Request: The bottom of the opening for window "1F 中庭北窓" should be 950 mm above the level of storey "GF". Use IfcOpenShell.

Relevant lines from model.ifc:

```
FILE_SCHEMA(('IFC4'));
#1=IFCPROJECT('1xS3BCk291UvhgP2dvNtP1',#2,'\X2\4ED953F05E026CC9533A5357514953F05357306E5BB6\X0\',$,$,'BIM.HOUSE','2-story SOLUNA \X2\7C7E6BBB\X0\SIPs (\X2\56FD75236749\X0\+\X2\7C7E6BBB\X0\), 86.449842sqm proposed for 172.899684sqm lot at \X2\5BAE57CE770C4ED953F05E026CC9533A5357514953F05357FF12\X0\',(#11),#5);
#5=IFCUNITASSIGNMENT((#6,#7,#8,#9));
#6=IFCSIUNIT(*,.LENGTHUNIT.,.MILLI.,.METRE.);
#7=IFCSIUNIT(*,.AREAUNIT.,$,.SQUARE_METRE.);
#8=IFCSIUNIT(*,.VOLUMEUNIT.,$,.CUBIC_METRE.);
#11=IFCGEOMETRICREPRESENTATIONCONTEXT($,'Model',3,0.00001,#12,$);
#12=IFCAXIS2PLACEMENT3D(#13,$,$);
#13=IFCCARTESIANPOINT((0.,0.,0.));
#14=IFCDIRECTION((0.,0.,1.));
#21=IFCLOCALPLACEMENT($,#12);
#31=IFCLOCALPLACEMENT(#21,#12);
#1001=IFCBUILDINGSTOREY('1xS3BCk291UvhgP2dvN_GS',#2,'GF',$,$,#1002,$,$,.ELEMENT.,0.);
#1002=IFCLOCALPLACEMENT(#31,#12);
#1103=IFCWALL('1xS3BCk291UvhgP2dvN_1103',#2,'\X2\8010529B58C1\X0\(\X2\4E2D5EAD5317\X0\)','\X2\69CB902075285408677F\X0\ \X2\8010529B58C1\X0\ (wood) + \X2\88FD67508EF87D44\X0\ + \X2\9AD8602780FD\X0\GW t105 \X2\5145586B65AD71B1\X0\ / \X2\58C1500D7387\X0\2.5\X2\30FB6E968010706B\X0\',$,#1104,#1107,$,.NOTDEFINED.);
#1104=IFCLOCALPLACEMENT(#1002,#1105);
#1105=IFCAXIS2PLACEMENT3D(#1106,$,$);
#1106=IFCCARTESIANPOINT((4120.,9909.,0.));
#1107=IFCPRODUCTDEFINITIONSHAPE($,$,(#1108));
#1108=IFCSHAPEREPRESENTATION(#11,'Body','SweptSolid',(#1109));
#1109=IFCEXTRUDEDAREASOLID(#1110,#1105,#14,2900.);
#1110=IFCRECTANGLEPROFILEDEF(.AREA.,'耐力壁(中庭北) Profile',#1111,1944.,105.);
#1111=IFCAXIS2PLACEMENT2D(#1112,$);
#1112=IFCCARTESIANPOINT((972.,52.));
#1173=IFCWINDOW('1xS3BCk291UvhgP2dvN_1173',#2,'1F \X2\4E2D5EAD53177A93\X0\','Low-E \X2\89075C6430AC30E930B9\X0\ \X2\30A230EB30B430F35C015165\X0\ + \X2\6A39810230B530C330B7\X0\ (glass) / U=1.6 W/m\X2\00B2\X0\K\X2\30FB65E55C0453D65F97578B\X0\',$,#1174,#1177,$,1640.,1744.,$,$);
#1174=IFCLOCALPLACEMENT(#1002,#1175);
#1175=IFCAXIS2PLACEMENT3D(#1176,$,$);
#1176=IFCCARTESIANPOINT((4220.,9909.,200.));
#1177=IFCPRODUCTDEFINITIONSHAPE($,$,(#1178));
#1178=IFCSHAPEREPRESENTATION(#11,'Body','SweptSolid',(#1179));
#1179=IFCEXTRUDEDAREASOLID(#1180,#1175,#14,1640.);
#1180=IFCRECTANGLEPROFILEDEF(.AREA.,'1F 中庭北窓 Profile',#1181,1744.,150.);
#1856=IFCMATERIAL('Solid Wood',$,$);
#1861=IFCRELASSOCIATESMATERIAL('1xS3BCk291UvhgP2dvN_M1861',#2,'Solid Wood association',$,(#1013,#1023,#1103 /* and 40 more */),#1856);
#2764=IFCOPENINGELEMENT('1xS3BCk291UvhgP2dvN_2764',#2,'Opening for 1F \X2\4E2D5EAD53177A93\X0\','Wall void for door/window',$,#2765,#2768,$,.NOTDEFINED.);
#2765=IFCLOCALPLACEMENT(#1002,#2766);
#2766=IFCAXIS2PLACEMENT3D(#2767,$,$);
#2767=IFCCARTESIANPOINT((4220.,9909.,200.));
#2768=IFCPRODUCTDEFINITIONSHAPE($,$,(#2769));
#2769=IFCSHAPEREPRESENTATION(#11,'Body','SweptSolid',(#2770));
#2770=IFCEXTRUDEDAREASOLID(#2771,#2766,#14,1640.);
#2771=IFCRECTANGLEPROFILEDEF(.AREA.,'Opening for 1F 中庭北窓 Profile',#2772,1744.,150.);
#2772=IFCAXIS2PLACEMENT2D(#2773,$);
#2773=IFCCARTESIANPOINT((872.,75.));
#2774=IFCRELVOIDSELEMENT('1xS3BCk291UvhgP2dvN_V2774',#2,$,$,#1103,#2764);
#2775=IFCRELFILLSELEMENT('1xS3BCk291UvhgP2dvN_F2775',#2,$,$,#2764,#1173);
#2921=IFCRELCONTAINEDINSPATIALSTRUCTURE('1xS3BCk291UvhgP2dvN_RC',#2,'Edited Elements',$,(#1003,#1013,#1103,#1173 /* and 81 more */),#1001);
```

```python
import numpy as np
import ifcopenshell
import ifcopenshell.api.geometry
import ifcopenshell.geom
import ifcopenshell.util.element
import ifcopenshell.util.placement
import ifcopenshell.util.shape
import ifcopenshell.util.unit

model = ifcopenshell.open("model.ifc")
unit_scale = ifcopenshell.util.unit.calculate_unit_scale(model)

window = model.by_guid("1xS3BCk291UvhgP2dvN_1173")
opening = window.FillsVoids[0].RelatingOpeningElement
storey = ifcopenshell.util.element.get_container(window, ifc_class="IfcBuildingStorey")
level = ifcopenshell.util.placement.get_local_placement(storey.ObjectPlacement)[2, 3]

# The opening's origin need not be at the sill, so measure its lowest point.
shape = ifcopenshell.geom.create_shape(ifcopenshell.geom.settings(), opening)
bottom = ifcopenshell.util.shape.get_shape_bottom_elevation(shape, shape.geometry) / unit_scale
dz = level + 0.95 / unit_scale - bottom

shift = np.array([0.0, 0.0, dz])
# The window is not placed relative to its opening, so move both.
for product in (opening, window):
    matrix = ifcopenshell.util.placement.get_local_placement(product.ObjectPlacement)
    matrix[:3, 3] += shift
    ifcopenshell.api.geometry.edit_object_placement(model, product=product, matrix=matrix, is_si=False)

print(f"moved by {dz * unit_scale:+.3f} m")

model.write("model-out.ifc")
```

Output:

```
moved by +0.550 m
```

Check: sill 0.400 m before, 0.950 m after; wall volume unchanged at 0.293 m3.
